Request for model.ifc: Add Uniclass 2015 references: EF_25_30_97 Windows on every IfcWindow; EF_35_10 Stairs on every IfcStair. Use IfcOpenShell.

First a look at what the model holds.

```python
import ifcopenshell

model = ifcopenshell.open("model.ifc")
print(model.schema)
print("classifications:", [c.Name for c in model.by_type("IfcClassification")])
for ifc_class in ("IfcDoor", "IfcRoof", "IfcStair", "IfcWall", "IfcWindow"):
    print(ifc_class, len(model.by_type(ifc_class)))
```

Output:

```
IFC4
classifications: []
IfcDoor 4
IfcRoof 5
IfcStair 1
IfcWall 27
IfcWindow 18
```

```python
import ifcopenshell
import ifcopenshell.api.classification

model = ifcopenshell.open("model.ifc")

system = ifcopenshell.api.classification.add_classification(model, classification="Uniclass 2015")

codes = {
    "IfcWindow": ("EF_25_30_97", "Windows"),
    "IfcStair": ("EF_35_10", "Stairs"),
}
for ifc_class, (code, name) in codes.items():
    products = model.by_type(ifc_class)
    ifcopenshell.api.classification.add_reference(
        model, products=products, classification=system, identification=code, name=name
    )
    print(code, len(products))

model.write("model_rev.ifc")
```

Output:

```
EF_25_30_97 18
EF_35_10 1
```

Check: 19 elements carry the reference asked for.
